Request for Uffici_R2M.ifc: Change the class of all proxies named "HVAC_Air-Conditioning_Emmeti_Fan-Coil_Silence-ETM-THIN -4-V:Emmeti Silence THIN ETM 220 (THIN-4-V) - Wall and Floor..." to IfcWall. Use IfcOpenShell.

First a look at what the model holds.

```python
import re

import ifcopenshell

model = ifcopenshell.open("Uffici_R2M.ifc")
print(model.schema)
seen = {}
for e in model.by_type("IfcBuildingElementProxy"):
    name = re.sub(r":\d+(:\d+)?$", "", e.Name or "")  # drop the element id that some exporters append
    seen[name] = seen.get(name, 0) + 1
for name, count in sorted(seen.items()):
    print(count, "x", name)
```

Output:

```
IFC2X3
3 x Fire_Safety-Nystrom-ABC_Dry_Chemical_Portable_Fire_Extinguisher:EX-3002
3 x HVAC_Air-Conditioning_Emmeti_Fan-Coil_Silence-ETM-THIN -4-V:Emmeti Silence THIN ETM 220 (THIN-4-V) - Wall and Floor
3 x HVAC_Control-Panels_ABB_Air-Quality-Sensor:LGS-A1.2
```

```python
import ifcopenshell
import ifcopenshell.api.root

model = ifcopenshell.open("Uffici_R2M.ifc")

proxies = [e.id() for e in model.by_type("IfcBuildingElementProxy") if (e.Name or "").startswith("HVAC_Air-Conditioning_Emmeti_Fan-Coil_Silence-ETM-THIN -4-V:Emmeti Silence THIN ETM 220 (THIN-4-V) - Wall and Floor")]
for step_id in proxies:
    proxy = model.by_id(step_id)
    # Reclassifying a typed element also reclassifies its type and the type's other occurrences.
    if proxy.is_a("IfcBuildingElementProxy"):
        ifcopenshell.api.root.reassign_class(model, product=proxy, ifc_class="IfcWall")

print(sum(model.by_id(i).is_a("IfcWall") for i in proxies), "reclassified")

model.write("Uffici_R2M_updated.ifc")
```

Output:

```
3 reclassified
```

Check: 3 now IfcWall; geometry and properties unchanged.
